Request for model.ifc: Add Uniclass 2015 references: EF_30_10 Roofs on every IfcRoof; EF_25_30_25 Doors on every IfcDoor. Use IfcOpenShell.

First a look at what the model holds.

```python
import ifcopenshell

model = ifcopenshell.open("model.ifc")
print(model.schema)
print("classifications:", [c.Name for c in model.by_type("IfcClassification")])
for ifc_class in ("IfcDoor", "IfcRoof", "IfcStair", "IfcWall", "IfcWindow"):
    print(ifc_class, len(model.by_type(ifc_class)))
```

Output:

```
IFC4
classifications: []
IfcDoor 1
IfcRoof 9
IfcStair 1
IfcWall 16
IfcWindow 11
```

```python
import ifcopenshell
import ifcopenshell.api.classification

model = ifcopenshell.open("model.ifc")

system = ifcopenshell.api.classification.add_classification(model, classification="Uniclass 2015")

codes = {
    "IfcRoof": ("EF_30_10", "Roofs"),
    "IfcDoor": ("EF_25_30_25", "Doors"),
}
for ifc_class, (code, name) in codes.items():
    products = model.by_type(ifc_class)
    ifcopenshell.api.classification.add_reference(
        model, products=products, classification=system, identification=code, name=name
    )
    print(code, len(products))

model.write("model_edited.ifc")
```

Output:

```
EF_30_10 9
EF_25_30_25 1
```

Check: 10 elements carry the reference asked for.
